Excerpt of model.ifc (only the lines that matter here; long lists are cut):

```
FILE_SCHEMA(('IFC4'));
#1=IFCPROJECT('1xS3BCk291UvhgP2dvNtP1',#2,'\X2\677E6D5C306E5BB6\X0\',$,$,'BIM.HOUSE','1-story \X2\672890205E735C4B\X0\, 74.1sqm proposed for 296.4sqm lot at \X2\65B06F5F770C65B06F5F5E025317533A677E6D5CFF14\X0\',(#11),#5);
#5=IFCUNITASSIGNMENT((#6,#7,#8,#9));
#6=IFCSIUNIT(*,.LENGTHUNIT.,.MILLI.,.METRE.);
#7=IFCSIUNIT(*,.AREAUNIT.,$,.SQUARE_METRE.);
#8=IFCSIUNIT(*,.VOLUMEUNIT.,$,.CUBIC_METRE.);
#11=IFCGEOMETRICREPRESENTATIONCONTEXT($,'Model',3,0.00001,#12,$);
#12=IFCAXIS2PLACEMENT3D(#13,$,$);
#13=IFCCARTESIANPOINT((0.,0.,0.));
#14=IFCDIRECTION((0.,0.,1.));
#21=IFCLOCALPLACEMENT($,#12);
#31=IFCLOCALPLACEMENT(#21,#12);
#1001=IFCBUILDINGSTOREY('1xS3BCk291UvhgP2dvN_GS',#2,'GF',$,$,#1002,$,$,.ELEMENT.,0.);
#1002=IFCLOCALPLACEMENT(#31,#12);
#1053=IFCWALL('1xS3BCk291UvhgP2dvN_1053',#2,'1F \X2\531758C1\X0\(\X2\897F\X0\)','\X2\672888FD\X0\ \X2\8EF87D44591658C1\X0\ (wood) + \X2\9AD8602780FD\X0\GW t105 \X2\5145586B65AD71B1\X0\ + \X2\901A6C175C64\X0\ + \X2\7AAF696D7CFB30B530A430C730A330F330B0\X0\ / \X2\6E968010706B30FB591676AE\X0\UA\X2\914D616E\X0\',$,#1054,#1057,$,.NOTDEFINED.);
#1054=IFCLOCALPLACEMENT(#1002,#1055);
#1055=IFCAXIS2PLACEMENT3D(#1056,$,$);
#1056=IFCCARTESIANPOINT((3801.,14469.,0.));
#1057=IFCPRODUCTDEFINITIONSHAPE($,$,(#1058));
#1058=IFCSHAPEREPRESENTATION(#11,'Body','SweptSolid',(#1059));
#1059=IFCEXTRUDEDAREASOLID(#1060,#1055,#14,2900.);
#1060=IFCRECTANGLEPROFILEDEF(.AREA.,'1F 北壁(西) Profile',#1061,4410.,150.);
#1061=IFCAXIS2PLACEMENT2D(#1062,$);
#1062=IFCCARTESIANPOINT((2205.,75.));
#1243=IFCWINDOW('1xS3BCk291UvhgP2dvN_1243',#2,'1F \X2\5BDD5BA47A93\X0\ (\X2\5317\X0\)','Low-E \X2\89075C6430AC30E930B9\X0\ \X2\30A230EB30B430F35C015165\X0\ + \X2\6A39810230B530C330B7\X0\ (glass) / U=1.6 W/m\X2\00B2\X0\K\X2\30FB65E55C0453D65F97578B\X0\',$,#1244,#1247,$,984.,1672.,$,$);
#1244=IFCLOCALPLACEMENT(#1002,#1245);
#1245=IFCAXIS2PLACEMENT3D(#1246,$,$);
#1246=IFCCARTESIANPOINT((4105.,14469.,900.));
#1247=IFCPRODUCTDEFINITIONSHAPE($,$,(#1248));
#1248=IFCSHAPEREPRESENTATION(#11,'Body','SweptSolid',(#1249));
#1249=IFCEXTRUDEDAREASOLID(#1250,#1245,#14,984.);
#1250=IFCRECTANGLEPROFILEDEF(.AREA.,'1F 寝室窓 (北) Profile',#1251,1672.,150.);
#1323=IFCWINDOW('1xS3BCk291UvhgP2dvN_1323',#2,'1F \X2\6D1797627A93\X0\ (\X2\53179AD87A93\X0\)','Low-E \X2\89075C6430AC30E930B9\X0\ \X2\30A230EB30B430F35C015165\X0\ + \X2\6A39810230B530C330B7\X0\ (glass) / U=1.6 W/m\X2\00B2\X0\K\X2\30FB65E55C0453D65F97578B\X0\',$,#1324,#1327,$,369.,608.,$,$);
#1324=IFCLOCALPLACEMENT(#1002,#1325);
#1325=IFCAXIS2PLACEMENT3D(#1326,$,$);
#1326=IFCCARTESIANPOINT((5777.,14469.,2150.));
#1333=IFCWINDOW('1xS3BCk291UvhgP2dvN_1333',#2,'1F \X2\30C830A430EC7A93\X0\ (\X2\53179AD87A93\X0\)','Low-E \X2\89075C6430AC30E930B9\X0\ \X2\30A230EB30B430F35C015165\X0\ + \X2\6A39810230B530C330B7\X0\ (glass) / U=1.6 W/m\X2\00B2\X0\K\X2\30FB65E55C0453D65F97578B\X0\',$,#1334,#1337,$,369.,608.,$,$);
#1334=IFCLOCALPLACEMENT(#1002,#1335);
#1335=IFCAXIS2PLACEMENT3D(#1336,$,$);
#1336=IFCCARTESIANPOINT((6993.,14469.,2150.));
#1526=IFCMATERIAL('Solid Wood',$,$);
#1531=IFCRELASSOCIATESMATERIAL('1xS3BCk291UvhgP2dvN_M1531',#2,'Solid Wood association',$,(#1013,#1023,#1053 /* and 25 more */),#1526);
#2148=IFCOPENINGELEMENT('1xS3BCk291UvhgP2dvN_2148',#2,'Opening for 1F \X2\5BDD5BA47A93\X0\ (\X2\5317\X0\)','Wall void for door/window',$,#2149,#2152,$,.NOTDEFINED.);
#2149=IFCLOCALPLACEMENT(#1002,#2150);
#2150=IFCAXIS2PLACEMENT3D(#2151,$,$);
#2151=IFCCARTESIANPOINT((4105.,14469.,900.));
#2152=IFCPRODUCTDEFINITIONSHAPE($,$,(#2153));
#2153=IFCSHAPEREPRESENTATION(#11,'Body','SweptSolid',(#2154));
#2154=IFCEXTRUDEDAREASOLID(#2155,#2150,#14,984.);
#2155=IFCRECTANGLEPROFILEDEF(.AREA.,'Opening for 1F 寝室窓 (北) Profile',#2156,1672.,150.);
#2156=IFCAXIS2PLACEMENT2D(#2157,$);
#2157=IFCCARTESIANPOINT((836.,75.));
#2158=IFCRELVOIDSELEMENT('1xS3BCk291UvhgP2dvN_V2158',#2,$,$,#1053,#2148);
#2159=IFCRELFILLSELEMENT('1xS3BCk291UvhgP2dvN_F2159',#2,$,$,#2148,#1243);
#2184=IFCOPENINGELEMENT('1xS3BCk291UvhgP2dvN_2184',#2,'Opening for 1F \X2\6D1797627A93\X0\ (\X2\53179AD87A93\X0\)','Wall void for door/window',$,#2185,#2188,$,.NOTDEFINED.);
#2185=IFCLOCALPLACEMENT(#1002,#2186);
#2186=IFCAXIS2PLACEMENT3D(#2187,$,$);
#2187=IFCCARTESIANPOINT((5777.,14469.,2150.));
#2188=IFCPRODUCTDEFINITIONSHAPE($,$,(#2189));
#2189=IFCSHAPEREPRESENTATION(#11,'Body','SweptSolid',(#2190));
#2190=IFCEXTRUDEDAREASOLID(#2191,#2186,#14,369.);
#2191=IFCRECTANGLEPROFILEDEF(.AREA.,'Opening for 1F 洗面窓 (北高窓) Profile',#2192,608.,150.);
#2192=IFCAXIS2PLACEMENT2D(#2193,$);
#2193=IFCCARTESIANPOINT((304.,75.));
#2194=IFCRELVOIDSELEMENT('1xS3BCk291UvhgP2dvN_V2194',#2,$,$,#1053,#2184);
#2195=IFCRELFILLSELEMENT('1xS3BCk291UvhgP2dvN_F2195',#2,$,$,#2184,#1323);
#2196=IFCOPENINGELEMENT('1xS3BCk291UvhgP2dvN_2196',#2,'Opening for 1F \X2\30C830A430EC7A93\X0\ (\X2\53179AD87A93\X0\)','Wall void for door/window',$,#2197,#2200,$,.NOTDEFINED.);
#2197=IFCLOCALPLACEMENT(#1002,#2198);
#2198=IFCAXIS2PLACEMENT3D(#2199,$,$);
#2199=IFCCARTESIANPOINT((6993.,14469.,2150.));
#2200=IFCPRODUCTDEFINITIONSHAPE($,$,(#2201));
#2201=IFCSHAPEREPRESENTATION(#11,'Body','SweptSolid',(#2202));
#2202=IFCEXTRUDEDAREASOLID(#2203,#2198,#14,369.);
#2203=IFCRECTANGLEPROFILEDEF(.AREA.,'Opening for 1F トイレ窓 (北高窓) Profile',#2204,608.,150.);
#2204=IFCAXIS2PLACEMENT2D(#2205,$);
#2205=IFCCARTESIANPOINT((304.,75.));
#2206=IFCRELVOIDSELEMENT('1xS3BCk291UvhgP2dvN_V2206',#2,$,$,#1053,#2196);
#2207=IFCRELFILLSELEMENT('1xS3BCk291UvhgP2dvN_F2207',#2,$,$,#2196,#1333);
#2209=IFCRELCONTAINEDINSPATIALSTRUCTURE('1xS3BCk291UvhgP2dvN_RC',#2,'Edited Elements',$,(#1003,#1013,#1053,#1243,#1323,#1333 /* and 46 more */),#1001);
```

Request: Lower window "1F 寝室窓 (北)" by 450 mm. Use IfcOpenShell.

```python
import numpy as np
import ifcopenshell
import ifcopenshell.api.geometry
import ifcopenshell.util.placement
import ifcopenshell.util.unit

model = ifcopenshell.open("model.ifc")
unit_scale = ifcopenshell.util.unit.calculate_unit_scale(model)

window = model.by_guid("1xS3BCk291UvhgP2dvN_1243")
opening = window.FillsVoids[0].RelatingOpeningElement
dz = -0.45 / unit_scale

shift = np.array([0.0, 0.0, dz])
# The window is not placed relative to its opening, so move both.
for product in (opening, window):
    matrix = ifcopenshell.util.placement.get_local_placement(product.ObjectPlacement)
    matrix[:3, 3] += shift
    ifcopenshell.api.geometry.edit_object_placement(model, product=product, matrix=matrix, is_si=False)

print(f"moved by {dz * unit_scale:+.3f} m")

model.write("model_updated.ifc")
```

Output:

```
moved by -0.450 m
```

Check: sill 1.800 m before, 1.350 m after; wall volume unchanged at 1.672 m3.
